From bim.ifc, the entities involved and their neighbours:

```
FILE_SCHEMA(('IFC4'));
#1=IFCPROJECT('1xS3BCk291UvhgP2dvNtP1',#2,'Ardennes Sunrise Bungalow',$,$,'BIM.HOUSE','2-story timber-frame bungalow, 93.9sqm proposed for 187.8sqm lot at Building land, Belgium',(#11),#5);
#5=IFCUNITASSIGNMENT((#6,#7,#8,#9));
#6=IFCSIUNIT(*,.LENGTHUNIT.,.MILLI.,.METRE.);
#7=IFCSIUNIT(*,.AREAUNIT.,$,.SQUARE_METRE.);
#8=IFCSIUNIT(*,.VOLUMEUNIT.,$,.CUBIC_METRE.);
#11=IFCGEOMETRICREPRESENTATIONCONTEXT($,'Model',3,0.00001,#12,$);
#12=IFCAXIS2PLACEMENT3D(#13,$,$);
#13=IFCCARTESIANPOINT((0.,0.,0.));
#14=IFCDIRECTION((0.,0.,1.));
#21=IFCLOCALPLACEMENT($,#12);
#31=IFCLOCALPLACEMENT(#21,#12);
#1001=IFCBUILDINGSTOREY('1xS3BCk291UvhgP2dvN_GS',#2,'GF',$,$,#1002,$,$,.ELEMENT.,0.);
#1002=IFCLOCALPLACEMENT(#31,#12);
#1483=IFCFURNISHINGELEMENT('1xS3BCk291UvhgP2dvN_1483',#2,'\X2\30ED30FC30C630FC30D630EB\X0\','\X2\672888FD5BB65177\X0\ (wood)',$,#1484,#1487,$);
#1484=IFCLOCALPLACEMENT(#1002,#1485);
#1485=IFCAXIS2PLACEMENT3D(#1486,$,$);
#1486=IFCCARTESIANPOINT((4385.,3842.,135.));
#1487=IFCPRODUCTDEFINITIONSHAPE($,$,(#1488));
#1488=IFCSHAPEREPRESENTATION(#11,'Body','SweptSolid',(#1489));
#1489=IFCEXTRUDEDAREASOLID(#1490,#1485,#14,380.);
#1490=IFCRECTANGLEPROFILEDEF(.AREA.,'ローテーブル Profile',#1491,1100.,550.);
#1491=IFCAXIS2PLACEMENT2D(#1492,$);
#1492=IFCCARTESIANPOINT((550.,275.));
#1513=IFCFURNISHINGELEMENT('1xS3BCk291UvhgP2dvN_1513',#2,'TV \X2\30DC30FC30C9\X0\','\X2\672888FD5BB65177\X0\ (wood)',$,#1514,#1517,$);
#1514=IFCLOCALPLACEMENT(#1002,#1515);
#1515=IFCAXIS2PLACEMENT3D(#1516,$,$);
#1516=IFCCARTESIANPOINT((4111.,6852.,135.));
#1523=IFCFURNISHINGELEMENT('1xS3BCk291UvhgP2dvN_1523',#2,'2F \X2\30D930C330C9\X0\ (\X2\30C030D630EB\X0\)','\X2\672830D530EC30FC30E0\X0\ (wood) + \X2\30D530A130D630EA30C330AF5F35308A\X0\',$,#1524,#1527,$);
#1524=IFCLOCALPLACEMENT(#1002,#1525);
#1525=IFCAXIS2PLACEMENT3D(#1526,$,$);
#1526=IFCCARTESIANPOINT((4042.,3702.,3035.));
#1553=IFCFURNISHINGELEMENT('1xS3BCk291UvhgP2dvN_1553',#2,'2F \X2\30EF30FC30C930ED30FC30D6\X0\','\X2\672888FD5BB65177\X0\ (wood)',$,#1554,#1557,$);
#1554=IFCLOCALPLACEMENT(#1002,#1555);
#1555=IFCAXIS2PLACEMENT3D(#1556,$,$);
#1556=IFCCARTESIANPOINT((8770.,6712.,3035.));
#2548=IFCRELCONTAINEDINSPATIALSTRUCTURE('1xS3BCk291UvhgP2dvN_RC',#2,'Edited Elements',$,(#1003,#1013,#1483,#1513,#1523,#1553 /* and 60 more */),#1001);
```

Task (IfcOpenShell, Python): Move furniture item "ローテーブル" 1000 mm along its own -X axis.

```python
import ifcopenshell
import ifcopenshell.api.geometry
import ifcopenshell.util.placement

model = ifcopenshell.open("bim.ifc")

item = model.by_guid("1xS3BCk291UvhgP2dvN_1483")
matrix = ifcopenshell.util.placement.get_local_placement(item.ObjectPlacement)
matrix[:3, 3] -= matrix[:3, 0] * 1000.0
ifcopenshell.api.geometry.edit_object_placement(model, product=item, matrix=matrix, is_si=False)

print(ifcopenshell.util.placement.get_local_placement(item.ObjectPlacement).round(3) + 0.0)

model.write("bim_edited.ifc")
```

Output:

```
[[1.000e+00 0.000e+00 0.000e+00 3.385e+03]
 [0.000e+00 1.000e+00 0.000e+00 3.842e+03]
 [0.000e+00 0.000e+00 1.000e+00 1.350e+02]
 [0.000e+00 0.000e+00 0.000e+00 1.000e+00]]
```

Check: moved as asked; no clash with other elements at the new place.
